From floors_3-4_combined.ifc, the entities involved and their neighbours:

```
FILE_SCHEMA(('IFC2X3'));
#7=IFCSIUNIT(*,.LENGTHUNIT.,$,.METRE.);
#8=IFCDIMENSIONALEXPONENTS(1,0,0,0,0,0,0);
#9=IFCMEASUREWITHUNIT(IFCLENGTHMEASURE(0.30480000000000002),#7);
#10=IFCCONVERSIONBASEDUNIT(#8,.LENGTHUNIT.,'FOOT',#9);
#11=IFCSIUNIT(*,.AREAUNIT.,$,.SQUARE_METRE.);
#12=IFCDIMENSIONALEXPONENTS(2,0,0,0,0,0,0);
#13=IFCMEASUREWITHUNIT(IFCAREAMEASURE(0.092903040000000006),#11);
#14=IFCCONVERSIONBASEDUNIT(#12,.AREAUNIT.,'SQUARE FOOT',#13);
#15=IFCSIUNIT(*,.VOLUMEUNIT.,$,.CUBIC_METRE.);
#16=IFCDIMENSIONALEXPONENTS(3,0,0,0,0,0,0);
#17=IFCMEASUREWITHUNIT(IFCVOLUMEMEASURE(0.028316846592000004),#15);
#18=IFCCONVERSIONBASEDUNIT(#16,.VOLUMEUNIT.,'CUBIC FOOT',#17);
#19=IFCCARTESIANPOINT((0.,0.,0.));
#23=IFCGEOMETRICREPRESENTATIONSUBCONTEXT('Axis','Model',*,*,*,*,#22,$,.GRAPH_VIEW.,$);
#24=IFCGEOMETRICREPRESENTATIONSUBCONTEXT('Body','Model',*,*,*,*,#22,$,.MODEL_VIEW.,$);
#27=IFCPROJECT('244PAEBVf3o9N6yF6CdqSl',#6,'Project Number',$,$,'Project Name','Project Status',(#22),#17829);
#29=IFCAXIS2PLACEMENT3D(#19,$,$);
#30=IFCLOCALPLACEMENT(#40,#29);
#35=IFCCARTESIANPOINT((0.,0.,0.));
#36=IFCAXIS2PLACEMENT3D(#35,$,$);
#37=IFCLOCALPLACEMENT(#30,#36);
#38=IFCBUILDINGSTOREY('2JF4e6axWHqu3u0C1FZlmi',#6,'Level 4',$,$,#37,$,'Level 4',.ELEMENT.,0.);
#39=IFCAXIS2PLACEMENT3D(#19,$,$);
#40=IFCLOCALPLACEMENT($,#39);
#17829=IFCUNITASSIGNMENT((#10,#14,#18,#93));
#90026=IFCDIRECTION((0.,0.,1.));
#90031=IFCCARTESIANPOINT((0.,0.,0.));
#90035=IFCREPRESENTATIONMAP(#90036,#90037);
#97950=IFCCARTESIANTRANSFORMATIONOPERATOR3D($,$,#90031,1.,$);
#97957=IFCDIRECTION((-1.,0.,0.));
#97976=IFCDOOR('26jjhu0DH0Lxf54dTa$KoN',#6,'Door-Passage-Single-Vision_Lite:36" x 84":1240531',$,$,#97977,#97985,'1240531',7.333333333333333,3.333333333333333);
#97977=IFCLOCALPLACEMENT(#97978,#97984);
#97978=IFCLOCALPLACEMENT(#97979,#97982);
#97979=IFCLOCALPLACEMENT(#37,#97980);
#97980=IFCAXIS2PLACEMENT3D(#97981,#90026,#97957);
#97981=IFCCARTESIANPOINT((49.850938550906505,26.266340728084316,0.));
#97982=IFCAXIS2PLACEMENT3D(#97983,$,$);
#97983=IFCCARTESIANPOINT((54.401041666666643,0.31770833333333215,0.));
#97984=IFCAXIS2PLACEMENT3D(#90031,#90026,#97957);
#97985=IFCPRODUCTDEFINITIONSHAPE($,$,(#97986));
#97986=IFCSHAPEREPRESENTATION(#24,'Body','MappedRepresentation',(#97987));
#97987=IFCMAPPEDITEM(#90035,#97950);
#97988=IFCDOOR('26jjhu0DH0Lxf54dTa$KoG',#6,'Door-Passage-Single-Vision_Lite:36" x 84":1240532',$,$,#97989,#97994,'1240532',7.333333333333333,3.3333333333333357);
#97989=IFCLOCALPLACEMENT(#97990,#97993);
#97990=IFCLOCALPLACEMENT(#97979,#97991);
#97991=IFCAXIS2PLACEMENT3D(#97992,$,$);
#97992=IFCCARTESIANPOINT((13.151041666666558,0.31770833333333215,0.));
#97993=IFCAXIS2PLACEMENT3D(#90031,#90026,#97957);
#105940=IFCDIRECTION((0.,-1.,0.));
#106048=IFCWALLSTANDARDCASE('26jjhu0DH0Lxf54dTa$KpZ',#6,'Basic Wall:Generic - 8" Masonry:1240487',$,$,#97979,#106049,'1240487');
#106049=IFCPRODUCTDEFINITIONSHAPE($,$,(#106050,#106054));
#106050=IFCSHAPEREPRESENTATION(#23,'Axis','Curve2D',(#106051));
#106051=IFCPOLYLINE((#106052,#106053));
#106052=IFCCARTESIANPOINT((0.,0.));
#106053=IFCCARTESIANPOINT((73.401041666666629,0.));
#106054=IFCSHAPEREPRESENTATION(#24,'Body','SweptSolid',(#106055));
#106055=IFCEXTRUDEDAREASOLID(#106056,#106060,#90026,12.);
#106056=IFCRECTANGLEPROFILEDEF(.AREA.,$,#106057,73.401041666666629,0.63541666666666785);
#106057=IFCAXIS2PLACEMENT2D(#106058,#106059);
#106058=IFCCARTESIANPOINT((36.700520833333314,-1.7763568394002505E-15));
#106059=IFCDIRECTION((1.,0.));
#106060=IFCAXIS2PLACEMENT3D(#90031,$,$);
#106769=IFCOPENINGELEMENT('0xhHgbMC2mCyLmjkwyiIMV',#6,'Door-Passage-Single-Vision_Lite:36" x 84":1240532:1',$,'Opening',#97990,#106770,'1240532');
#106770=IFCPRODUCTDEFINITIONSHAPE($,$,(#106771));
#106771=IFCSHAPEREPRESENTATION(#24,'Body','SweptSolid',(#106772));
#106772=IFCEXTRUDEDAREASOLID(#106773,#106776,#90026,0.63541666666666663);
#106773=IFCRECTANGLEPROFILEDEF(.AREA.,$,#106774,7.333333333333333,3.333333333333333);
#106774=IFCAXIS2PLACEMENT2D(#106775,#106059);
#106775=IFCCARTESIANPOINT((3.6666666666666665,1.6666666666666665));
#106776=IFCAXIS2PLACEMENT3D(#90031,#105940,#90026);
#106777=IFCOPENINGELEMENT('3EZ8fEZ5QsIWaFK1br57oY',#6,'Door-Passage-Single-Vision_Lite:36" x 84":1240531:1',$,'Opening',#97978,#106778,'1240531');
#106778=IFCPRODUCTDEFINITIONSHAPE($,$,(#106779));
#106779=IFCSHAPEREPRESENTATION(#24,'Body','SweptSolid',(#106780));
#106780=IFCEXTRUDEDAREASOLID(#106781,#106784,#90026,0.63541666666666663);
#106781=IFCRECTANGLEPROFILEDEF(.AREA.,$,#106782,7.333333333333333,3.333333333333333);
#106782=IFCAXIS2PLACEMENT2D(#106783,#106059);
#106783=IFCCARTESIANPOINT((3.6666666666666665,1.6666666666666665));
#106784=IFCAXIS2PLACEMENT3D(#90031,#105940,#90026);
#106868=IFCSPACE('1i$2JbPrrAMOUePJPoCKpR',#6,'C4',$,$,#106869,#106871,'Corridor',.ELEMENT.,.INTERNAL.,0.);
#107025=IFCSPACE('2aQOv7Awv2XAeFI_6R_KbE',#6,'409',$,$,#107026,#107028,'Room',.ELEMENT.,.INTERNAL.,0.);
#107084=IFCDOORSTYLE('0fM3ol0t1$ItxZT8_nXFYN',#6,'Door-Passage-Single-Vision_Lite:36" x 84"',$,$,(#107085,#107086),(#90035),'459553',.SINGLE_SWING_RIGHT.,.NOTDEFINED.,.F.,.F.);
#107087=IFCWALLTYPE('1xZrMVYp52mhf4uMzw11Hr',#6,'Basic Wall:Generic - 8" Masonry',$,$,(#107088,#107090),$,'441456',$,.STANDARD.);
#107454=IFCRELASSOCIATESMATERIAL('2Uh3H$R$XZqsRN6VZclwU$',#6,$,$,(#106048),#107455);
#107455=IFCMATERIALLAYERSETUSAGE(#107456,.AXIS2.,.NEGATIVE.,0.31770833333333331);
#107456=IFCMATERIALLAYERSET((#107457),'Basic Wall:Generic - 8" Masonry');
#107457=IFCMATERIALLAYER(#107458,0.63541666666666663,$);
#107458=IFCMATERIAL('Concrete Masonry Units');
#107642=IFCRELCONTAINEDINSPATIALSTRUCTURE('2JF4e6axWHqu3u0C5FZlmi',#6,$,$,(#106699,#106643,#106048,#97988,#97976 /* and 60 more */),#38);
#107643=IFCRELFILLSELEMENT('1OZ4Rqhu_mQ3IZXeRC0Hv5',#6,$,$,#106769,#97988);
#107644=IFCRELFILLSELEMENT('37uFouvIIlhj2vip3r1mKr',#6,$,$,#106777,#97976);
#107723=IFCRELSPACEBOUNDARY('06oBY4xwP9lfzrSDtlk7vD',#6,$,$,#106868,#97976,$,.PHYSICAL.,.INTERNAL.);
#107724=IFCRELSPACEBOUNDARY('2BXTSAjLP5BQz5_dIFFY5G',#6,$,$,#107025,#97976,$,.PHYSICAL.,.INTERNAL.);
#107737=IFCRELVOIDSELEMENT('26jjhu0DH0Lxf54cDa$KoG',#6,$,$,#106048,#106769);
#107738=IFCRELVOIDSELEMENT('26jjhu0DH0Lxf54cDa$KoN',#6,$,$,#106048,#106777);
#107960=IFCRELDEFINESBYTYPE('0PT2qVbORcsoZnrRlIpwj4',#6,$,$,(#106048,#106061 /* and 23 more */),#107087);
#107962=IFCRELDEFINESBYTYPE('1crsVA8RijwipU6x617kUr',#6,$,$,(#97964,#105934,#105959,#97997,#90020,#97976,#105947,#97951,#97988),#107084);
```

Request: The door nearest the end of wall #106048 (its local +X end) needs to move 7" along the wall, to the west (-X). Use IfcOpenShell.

```python
import ifcopenshell
import ifcopenshell.api.geometry
import ifcopenshell.util.placement
import ifcopenshell.util.unit

model = ifcopenshell.open("floors_3-4_combined.ifc")
unit_scale = ifcopenshell.util.unit.calculate_unit_scale(model)

door = model.by_guid("26jjhu0DH0Lxf54dTa$KoN")
opening = door.FillsVoids[0].RelatingOpeningElement
wall = opening.VoidsElements[0].RelatingBuildingElement

wall_matrix = ifcopenshell.util.placement.get_local_placement(wall.ObjectPlacement)
shift = wall_matrix[:3, 0] * 7 * 0.0254 / unit_scale
before = ifcopenshell.util.placement.get_local_placement(door.ObjectPlacement)[:3, 3].copy()

# The door is placed relative to its opening, so it follows when the opening moves.
matrix = ifcopenshell.util.placement.get_local_placement(opening.ObjectPlacement)
matrix[:3, 3] += shift
ifcopenshell.api.geometry.edit_object_placement(
    model, product=opening, matrix=matrix, is_si=False, should_transform_children=True
)

after = ifcopenshell.util.placement.get_local_placement(door.ObjectPlacement)[:3, 3]
print("door moved by", (after - before).round(3) + 0.0)

model.write("floors_3-4_combined_edited.ifc")
```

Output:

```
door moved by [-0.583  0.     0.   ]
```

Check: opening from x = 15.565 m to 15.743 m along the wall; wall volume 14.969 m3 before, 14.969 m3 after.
